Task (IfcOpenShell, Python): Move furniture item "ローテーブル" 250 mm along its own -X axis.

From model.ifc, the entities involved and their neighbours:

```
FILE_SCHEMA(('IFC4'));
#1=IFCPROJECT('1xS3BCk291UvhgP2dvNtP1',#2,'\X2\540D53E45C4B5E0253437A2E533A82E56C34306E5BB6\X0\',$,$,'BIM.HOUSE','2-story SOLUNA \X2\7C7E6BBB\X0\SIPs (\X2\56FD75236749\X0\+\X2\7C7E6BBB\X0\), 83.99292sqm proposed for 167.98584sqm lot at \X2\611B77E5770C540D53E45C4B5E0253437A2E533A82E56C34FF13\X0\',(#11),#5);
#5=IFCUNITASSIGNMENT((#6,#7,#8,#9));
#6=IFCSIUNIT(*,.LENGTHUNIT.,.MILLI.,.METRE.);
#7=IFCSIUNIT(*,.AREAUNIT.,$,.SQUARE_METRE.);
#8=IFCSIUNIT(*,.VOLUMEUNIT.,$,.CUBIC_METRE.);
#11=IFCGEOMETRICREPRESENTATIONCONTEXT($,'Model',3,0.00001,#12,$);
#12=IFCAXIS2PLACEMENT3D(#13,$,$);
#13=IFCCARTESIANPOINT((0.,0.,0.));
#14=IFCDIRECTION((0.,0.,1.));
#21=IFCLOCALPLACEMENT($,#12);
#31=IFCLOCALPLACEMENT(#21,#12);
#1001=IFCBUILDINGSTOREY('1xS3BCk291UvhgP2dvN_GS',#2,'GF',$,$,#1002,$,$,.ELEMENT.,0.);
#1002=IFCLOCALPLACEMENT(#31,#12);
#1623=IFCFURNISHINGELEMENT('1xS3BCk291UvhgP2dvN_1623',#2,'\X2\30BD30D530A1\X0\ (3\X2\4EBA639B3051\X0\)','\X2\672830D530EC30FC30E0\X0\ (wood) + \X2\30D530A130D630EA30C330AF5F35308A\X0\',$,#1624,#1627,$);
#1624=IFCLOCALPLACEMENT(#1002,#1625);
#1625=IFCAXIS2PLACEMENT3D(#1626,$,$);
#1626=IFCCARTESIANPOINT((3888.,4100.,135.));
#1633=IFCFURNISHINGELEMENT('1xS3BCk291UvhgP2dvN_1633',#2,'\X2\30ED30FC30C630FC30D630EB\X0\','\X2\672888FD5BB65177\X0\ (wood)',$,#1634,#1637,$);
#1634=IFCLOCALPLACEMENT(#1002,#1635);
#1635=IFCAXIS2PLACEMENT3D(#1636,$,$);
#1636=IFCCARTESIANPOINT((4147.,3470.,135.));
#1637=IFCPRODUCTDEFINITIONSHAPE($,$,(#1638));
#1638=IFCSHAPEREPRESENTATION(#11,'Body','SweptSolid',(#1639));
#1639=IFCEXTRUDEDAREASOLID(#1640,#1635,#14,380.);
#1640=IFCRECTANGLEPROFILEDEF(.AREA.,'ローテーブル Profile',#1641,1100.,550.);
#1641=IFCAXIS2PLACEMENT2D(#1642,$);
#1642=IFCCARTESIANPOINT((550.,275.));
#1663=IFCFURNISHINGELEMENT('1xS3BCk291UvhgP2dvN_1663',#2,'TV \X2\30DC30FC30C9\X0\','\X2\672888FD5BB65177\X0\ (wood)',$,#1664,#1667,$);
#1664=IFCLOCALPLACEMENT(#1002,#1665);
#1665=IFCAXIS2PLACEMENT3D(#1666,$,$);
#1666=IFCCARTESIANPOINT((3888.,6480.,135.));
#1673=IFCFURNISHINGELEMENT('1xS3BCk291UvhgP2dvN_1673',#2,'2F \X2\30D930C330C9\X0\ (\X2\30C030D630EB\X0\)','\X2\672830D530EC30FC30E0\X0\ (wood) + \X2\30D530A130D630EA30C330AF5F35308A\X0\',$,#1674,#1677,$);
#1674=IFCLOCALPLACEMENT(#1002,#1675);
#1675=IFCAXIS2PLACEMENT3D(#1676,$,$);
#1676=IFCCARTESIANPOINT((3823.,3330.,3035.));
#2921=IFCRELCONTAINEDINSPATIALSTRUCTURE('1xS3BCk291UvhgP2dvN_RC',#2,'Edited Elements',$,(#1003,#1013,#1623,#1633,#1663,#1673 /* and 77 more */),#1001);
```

```python
import ifcopenshell
import ifcopenshell.api.geometry
import ifcopenshell.util.placement

model = ifcopenshell.open("model.ifc")

item = model.by_guid("1xS3BCk291UvhgP2dvN_1633")
matrix = ifcopenshell.util.placement.get_local_placement(item.ObjectPlacement)
matrix[:3, 3] -= matrix[:3, 0] * 250.0
ifcopenshell.api.geometry.edit_object_placement(model, product=item, matrix=matrix, is_si=False)

print(ifcopenshell.util.placement.get_local_placement(item.ObjectPlacement).round(3) + 0.0)

model.write("model_edited.ifc")
```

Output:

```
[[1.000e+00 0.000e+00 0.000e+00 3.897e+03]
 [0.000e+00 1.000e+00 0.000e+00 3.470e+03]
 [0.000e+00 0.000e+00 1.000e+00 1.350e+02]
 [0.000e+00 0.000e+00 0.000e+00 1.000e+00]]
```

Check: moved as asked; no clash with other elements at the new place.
